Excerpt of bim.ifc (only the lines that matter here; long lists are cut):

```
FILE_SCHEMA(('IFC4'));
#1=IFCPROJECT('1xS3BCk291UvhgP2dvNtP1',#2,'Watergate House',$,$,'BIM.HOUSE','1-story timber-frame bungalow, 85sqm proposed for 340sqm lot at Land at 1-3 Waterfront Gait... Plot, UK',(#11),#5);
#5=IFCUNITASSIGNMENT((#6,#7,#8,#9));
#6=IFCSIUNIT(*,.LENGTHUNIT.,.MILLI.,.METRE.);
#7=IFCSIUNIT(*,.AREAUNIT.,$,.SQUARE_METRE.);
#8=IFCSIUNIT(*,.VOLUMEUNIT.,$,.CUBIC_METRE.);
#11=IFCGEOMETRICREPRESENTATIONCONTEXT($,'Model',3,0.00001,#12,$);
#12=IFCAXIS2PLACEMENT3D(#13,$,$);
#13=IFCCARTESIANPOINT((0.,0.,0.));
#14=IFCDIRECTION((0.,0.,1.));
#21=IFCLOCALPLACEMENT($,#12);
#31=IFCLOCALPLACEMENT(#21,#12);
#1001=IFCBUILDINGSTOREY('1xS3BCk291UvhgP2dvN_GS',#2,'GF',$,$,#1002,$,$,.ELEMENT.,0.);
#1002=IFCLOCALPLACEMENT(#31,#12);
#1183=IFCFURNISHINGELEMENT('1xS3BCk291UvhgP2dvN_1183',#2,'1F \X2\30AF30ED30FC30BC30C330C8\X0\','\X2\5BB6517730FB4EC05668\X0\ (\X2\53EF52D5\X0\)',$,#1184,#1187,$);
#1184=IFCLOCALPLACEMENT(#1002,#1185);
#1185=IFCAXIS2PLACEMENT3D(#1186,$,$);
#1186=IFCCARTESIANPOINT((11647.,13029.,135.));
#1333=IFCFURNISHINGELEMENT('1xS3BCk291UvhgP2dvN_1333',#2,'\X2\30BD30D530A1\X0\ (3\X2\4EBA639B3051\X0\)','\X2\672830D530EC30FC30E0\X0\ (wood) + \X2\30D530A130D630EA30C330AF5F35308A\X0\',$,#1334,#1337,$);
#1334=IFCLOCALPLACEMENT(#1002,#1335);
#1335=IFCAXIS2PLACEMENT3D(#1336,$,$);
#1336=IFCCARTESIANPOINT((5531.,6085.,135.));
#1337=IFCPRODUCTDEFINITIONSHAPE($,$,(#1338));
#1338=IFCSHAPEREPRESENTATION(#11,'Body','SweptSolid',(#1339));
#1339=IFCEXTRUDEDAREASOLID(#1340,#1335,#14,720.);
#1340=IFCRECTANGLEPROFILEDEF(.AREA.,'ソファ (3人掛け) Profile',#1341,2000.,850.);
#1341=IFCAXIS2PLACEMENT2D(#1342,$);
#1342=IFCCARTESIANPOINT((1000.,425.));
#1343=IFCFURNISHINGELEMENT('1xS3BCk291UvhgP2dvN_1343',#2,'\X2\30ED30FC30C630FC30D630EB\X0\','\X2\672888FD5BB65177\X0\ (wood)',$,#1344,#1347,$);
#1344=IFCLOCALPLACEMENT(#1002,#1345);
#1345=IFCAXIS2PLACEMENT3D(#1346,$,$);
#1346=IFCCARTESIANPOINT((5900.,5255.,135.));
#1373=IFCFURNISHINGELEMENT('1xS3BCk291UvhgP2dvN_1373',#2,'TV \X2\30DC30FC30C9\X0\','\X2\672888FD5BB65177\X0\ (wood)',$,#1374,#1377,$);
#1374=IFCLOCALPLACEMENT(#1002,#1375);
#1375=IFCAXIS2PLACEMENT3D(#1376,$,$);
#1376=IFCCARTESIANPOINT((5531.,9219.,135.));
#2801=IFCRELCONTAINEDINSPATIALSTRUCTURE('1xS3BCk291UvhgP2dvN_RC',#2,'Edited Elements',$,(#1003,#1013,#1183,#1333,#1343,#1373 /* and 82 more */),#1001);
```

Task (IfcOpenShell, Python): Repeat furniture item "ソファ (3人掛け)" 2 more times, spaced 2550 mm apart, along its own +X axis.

```python
import ifcopenshell
import ifcopenshell.api.geometry
import ifcopenshell.api.root
import ifcopenshell.util.element
import ifcopenshell.util.placement
import ifcopenshell.util.unit

model = ifcopenshell.open("bim.ifc")
unit_scale = ifcopenshell.util.unit.calculate_unit_scale(model)


def reuse_history(source, copy):
    """copy_class also copies each property set's owner history, people and application; keep the originals."""
    for rel in copy.IsDefinedBy:
        if rel.is_a("IfcRelDefinesByProperties") and (history := rel.RelatingPropertyDefinition.OwnerHistory):
            rel.RelatingPropertyDefinition.OwnerHistory = source.OwnerHistory
            ifcopenshell.util.element.remove_deep2(model, history)


source = model.by_guid("1xS3BCk291UvhgP2dvN_1333")
base = ifcopenshell.util.placement.get_local_placement(source.ObjectPlacement)
step = base[:3, 0] * 2.55 / unit_scale

for i in range(1, 3):
    copy = ifcopenshell.api.root.copy_class(model, product=source)
    copy.Representation = ifcopenshell.util.element.copy_deep(
        model, source.Representation, exclude=["IfcGeometricRepresentationContext", "IfcRepresentationMap"]
    )
    reuse_history(source, copy)
    matrix = base.copy()
    matrix[:3, 3] += i * step
    print("added at", matrix[:3, 3].round(3) + 0.0)
    ifcopenshell.api.geometry.edit_object_placement(model, product=copy, matrix=matrix, is_si=False)

model.write("bim_v2.ifc")
```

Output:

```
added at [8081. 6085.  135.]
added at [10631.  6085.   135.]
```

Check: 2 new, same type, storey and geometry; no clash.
